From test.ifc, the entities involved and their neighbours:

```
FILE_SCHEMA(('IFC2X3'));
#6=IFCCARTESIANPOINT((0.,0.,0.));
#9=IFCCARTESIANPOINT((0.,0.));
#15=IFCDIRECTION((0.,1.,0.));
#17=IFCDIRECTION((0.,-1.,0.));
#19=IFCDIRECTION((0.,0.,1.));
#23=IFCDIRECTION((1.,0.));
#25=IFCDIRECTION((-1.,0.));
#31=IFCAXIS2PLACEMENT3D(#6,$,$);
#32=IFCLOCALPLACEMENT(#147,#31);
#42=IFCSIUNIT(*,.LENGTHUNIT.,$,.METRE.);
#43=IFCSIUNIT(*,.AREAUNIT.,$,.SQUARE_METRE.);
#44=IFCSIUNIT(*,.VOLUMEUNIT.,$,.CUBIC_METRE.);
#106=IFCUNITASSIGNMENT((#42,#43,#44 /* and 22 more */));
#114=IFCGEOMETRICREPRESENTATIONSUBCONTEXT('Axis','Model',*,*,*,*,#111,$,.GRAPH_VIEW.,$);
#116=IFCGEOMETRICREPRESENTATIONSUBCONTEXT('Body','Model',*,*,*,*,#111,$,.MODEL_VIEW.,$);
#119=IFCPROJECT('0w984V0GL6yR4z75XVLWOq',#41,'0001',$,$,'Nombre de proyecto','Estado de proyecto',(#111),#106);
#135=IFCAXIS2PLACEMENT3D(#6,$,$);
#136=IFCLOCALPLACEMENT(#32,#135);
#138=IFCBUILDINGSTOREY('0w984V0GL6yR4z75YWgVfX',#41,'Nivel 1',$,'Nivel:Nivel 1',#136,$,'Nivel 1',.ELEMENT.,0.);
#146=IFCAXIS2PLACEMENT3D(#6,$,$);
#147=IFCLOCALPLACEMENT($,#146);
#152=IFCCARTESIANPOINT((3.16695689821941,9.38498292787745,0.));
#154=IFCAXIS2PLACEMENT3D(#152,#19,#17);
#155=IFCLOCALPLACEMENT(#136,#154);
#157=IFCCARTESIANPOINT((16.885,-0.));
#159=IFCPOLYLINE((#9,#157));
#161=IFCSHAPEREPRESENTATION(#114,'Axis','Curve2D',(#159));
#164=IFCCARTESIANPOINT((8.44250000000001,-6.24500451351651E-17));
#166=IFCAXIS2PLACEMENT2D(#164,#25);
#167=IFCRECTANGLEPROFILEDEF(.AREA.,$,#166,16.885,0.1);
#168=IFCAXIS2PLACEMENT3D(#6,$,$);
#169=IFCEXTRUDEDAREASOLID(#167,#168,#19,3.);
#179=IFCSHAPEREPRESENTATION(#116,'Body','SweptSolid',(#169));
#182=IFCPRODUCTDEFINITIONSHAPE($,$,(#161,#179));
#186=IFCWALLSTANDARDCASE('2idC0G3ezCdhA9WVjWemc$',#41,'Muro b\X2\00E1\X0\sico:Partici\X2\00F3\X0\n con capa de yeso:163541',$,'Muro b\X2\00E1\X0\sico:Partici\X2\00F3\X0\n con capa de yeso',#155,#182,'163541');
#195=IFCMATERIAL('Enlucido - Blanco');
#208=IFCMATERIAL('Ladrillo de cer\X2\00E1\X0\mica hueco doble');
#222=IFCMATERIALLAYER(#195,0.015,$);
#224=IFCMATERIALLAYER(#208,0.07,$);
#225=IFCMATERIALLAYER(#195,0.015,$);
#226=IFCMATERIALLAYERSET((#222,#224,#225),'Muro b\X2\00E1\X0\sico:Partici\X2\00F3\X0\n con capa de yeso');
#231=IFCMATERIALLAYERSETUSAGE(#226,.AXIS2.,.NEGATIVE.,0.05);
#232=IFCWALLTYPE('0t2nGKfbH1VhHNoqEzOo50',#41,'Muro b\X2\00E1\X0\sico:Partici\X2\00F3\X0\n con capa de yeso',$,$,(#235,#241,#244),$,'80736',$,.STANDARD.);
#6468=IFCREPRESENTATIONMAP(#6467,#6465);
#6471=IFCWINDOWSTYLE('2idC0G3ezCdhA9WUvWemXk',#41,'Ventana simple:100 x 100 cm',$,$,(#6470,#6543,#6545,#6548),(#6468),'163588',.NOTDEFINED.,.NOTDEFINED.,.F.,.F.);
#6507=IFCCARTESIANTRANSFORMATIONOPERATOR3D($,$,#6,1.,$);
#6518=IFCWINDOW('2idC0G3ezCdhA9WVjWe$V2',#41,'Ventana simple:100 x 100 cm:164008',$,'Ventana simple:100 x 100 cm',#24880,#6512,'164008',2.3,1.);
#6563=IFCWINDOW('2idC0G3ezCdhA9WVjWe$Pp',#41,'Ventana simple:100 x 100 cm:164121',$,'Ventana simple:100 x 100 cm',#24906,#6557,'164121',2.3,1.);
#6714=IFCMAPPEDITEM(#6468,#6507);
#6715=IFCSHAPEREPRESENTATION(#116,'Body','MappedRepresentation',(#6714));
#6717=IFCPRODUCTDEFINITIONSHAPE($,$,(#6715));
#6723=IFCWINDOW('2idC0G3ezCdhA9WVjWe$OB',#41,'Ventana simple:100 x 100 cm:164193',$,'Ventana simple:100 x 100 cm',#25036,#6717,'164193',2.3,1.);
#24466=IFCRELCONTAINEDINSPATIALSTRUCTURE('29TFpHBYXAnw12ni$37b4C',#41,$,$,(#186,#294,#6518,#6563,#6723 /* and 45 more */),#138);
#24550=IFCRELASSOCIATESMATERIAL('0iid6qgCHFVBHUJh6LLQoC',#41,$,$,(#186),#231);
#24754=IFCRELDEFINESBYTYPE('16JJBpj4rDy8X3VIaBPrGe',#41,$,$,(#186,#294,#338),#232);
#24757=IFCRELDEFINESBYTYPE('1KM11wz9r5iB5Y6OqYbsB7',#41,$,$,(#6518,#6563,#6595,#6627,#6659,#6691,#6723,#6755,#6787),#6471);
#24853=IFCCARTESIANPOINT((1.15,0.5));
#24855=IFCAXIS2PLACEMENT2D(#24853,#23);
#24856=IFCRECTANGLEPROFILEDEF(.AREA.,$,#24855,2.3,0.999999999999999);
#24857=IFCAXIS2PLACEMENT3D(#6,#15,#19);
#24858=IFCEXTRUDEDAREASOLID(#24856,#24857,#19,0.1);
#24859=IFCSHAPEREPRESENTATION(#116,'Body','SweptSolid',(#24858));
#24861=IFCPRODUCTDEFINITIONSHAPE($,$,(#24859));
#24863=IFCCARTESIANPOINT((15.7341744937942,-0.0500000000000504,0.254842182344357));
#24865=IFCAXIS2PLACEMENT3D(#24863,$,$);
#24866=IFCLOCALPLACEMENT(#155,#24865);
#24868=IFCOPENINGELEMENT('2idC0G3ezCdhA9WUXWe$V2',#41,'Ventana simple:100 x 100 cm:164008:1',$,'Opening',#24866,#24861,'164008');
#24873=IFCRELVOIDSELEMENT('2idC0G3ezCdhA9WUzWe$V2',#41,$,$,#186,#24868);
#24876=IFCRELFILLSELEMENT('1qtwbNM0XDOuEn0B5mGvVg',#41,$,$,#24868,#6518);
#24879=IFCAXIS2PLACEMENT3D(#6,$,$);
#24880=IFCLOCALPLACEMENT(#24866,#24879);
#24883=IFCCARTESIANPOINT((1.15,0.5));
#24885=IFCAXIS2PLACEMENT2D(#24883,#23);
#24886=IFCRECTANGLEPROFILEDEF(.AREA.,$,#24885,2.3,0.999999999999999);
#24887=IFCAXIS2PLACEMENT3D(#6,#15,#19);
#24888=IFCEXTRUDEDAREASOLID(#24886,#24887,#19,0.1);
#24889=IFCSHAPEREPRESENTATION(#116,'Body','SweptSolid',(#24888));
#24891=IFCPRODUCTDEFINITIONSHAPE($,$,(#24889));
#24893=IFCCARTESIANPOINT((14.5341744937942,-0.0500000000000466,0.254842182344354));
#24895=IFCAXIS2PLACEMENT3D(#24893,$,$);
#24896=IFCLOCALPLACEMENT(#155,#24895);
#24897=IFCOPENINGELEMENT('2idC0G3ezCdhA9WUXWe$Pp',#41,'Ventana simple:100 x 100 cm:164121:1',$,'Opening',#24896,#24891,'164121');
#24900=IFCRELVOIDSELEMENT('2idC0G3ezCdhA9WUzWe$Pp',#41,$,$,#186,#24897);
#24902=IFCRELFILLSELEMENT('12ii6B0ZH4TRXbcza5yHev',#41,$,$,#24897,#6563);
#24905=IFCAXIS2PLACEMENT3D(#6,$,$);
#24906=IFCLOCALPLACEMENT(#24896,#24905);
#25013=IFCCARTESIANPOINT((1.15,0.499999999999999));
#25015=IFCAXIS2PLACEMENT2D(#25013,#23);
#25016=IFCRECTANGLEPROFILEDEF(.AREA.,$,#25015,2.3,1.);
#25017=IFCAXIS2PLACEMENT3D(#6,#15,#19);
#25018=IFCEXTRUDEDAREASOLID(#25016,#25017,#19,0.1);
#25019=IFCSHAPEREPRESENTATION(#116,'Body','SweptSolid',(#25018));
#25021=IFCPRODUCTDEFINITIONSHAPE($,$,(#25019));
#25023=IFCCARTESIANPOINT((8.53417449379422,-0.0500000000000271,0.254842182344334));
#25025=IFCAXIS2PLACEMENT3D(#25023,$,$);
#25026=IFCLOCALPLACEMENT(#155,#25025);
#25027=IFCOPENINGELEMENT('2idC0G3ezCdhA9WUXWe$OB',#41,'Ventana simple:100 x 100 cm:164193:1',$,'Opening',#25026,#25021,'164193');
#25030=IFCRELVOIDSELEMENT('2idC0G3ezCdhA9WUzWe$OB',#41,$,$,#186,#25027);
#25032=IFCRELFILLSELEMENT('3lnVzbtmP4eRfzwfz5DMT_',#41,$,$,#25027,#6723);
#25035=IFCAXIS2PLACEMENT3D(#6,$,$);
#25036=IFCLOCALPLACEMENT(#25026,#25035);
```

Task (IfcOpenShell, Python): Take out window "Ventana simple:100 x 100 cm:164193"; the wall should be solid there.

```python
import ifcopenshell
import ifcopenshell.api.feature
import ifcopenshell.api.root
import ifcopenshell.geom
import ifcopenshell.util.shape

model = ifcopenshell.open("test.ifc")
settings = ifcopenshell.geom.settings()


def volume(element):
    """Net volume in cubic metres, openings subtracted."""
    shape = ifcopenshell.geom.create_shape(settings, element)
    return ifcopenshell.util.shape.get_volume(shape.geometry)


window = model.by_guid("2idC0G3ezCdhA9WVjWe$OB")
opening = window.FillsVoids[0].RelatingOpeningElement
wall = opening.VoidsElements[0].RelatingBuildingElement
before = volume(wall)

ifcopenshell.api.root.remove_product(model, product=window)
ifcopenshell.api.feature.remove_feature(model, feature=opening)

after = volume(wall)

print(f"wall volume {before:.3f} -> {after:.3f} m3")

model.write("test_v2.ifc")
```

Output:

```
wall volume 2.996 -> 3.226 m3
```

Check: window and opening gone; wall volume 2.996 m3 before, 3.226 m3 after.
